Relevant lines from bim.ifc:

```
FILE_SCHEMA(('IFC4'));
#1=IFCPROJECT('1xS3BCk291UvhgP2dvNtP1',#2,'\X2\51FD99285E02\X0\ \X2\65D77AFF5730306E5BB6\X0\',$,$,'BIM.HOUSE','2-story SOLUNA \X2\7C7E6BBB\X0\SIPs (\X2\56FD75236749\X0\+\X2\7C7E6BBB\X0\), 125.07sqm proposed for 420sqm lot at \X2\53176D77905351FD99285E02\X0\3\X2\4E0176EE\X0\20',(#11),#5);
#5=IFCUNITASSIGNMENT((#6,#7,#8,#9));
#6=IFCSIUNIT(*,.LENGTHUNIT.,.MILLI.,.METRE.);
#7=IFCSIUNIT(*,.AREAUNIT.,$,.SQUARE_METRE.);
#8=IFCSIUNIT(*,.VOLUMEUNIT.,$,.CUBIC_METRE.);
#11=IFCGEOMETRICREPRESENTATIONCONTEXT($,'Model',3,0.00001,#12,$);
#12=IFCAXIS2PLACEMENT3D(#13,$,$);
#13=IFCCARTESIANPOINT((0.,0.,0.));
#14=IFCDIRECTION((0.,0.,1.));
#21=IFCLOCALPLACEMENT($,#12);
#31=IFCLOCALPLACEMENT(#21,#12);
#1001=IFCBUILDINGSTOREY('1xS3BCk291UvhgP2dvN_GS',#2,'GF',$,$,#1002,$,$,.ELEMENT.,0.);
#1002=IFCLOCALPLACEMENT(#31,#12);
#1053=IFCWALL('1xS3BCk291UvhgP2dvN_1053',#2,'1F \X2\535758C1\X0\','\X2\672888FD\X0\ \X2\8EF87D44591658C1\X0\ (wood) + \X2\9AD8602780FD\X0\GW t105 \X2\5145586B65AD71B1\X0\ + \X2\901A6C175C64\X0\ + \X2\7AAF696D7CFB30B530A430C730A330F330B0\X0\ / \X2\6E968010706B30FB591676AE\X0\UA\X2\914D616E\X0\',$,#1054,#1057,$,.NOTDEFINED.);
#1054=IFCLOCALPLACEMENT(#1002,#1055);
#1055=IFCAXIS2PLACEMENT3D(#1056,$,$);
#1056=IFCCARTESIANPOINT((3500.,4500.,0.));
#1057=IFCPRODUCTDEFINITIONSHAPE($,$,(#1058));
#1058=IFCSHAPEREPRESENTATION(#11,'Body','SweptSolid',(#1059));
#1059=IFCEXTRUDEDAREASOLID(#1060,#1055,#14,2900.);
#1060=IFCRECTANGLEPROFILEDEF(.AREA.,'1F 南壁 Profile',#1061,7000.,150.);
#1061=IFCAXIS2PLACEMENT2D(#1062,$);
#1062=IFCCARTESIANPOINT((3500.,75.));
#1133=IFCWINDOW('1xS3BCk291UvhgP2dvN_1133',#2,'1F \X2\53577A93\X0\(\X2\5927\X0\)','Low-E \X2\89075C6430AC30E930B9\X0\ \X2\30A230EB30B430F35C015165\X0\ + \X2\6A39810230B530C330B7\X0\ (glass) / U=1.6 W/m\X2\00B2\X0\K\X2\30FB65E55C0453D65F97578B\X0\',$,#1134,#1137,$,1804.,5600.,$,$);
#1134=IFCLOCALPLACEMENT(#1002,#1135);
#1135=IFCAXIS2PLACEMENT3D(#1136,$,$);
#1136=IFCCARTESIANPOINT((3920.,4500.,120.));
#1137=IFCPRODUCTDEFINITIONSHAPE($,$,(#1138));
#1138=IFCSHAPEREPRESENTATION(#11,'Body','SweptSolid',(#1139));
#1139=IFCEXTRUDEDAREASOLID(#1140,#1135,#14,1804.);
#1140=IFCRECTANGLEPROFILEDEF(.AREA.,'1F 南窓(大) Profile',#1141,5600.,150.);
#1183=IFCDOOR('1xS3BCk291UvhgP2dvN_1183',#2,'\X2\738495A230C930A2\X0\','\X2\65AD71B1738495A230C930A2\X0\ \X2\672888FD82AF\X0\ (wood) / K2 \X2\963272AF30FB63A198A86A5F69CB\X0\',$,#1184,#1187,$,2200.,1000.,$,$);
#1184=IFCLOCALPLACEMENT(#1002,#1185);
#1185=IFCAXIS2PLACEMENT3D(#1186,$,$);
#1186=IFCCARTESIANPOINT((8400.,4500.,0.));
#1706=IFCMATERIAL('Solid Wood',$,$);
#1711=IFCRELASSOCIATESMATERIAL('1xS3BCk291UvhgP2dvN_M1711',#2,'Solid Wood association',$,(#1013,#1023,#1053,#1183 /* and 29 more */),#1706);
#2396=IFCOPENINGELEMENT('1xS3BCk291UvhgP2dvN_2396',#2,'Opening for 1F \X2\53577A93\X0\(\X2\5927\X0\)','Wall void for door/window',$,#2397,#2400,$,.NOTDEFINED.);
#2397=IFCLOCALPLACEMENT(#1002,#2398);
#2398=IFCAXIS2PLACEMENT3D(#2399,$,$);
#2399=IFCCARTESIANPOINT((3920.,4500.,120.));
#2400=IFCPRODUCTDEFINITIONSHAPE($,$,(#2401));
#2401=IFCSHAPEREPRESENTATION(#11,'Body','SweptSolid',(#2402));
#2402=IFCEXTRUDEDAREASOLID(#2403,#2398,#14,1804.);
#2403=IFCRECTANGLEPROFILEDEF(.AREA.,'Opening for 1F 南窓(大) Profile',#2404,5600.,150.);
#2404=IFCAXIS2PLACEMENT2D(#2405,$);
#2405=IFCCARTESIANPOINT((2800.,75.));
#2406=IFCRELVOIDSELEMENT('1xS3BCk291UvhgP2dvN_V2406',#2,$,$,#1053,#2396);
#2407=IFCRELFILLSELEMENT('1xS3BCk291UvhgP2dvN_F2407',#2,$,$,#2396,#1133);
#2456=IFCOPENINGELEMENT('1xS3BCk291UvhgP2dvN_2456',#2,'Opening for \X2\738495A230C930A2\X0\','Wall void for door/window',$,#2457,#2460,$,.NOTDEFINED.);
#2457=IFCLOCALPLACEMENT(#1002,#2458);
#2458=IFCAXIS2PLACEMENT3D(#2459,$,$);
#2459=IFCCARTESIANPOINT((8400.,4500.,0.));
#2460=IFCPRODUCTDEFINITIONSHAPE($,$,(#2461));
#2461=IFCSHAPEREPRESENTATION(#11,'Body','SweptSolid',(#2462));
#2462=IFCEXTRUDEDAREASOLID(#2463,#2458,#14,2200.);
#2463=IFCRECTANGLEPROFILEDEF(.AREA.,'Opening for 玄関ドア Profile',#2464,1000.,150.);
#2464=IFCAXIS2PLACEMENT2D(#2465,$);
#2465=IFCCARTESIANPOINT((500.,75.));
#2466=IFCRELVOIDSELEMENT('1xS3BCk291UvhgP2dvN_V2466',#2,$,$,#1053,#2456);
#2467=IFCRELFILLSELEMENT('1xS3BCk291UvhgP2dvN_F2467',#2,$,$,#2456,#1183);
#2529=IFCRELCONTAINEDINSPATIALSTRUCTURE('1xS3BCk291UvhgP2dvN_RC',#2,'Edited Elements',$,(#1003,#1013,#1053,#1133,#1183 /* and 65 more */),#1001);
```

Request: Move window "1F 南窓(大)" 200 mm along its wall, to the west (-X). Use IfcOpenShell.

```python
import ifcopenshell
import ifcopenshell.api.geometry
import ifcopenshell.util.placement
import ifcopenshell.util.unit

model = ifcopenshell.open("bim.ifc")
unit_scale = ifcopenshell.util.unit.calculate_unit_scale(model)

window = model.by_guid("1xS3BCk291UvhgP2dvN_1133")
opening = window.FillsVoids[0].RelatingOpeningElement
wall = opening.VoidsElements[0].RelatingBuildingElement

wall_matrix = ifcopenshell.util.placement.get_local_placement(wall.ObjectPlacement)
shift = wall_matrix[:3, 0] * -0.2 / unit_scale
before = ifcopenshell.util.placement.get_local_placement(window.ObjectPlacement)[:3, 3].copy()

# The window is not placed relative to its opening, so move both.
for product in (opening, window):
    matrix = ifcopenshell.util.placement.get_local_placement(product.ObjectPlacement)
    matrix[:3, 3] += shift
    ifcopenshell.api.geometry.edit_object_placement(model, product=product, matrix=matrix, is_si=False)

after = ifcopenshell.util.placement.get_local_placement(window.ObjectPlacement)[:3, 3]
print("window moved by", (after - before).round(3) + 0.0)

model.write("bim_updated.ifc")
```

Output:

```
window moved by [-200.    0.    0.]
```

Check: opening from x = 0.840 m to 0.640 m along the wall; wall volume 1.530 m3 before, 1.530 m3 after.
